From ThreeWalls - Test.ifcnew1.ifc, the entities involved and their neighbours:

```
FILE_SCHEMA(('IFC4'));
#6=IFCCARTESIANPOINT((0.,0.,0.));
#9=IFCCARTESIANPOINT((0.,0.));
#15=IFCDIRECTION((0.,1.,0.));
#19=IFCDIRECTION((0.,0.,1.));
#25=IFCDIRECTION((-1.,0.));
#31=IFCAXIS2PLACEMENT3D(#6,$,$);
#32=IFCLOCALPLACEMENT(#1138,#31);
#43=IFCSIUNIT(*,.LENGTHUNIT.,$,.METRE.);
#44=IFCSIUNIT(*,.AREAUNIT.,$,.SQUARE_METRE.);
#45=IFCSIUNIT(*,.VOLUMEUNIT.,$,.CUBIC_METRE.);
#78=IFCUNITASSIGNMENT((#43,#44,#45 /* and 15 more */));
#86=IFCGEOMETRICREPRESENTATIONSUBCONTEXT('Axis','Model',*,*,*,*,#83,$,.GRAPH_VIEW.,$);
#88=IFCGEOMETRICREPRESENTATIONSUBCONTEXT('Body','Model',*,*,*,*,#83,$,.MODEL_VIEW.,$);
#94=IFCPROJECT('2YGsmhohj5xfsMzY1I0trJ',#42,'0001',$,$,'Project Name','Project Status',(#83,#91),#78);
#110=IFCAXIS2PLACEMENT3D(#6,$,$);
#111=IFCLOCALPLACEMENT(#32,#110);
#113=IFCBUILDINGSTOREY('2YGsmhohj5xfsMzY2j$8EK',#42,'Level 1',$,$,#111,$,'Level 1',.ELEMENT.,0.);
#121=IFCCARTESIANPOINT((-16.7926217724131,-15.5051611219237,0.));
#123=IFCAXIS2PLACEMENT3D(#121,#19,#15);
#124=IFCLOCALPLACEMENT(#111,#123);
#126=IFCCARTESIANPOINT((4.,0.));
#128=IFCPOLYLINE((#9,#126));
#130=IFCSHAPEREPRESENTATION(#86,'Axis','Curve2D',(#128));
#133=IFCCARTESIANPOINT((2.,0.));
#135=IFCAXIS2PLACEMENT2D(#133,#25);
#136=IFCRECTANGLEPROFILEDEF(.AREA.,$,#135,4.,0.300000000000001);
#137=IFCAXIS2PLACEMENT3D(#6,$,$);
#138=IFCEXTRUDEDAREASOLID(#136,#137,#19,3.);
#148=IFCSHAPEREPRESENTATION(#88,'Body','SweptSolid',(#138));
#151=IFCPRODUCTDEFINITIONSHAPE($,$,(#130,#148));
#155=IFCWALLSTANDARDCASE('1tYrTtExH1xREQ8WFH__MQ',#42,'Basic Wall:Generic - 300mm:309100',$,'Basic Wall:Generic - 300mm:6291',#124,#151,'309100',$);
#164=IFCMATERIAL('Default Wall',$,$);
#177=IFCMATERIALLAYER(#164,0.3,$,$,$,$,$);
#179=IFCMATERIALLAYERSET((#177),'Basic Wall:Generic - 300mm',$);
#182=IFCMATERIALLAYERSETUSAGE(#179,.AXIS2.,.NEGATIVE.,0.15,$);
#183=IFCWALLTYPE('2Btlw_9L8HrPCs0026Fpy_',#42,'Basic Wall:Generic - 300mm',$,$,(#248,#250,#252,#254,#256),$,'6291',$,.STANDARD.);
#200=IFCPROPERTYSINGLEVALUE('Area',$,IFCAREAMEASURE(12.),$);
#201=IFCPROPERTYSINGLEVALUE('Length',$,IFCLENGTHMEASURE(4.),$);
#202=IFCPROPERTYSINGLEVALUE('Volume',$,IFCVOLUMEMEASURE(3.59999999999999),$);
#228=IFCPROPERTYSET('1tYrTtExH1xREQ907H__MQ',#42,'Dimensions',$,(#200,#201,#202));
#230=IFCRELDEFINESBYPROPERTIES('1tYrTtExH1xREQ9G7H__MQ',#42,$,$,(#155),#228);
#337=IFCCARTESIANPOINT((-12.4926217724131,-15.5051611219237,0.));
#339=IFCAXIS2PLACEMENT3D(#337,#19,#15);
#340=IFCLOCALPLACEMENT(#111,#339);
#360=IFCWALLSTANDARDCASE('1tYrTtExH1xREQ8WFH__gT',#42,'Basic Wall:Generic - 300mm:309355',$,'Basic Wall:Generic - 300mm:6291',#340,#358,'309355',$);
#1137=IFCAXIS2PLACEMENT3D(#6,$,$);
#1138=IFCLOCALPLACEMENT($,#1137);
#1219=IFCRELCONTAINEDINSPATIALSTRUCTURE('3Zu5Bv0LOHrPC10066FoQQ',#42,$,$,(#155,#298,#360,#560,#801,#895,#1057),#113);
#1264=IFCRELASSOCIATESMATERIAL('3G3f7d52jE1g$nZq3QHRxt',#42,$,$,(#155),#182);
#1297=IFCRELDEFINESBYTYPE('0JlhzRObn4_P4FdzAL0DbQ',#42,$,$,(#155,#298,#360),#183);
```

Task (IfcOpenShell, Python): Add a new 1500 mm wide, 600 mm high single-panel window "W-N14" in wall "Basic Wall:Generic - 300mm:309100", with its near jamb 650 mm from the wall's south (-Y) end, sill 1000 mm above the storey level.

```python
import numpy as np
import ifcopenshell
import ifcopenshell.api.feature
import ifcopenshell.api.geometry
import ifcopenshell.api.pset
import ifcopenshell.api.root
import ifcopenshell.api.spatial
import ifcopenshell.geom
import ifcopenshell.util.element
import ifcopenshell.util.placement
import ifcopenshell.util.representation
import ifcopenshell.util.shape
import ifcopenshell.util.unit

model = ifcopenshell.open("ThreeWalls - Test.ifcnew1.ifc")
unit_scale = ifcopenshell.util.unit.calculate_unit_scale(model)
area_scale = ifcopenshell.util.unit.calculate_unit_scale(model, "AREAUNIT")
volume_scale = ifcopenshell.util.unit.calculate_unit_scale(model, "VOLUMEUNIT")
settings = ifcopenshell.geom.settings()


def volume(element):
    """Net volume in cubic metres, openings subtracted."""
    shape = ifcopenshell.geom.create_shape(settings, element)
    return ifcopenshell.util.shape.get_volume(shape.geometry)


wall = model.by_guid("1tYrTtExH1xREQ8WFH__MQ")
storey = ifcopenshell.util.element.get_container(wall, ifc_class="IfcBuildingStorey")
context = ifcopenshell.util.representation.get_context(model, "Model", "Body", "MODEL_VIEW")
before = volume(wall)

width, height, from_end, sill = 1.5, 0.6, 0.65, 1  # metres

# The wall runs along its own X axis, and the end named is its -X end.
wall_shape = ifcopenshell.geom.create_shape(settings, wall)
x, y, z = ifcopenshell.util.shape.get_vertices(wall_shape.geometry).T
start = x.min() + from_end
face, thickness = float(y.min()), float(y.max() - y.min())
wall_matrix = ifcopenshell.util.placement.get_local_placement(wall.ObjectPlacement)
level = ifcopenshell.util.placement.get_local_placement(storey.ObjectPlacement)[2, 3]


def in_wall(x, y):
    """Placement at x, y metres in the wall's axes, at sill height."""
    matrix = wall_matrix.copy()
    matrix[:, 3] = wall_matrix @ np.array([x / unit_scale, y / unit_scale, 0.0, 1.0])
    matrix[2, 3] = level + sill / unit_scale
    return matrix


# Opening: a box that overshoots both wall faces by 50 mm.
opening = ifcopenshell.api.root.create_entity(model, ifc_class="IfcOpeningElement", predefined_type="OPENING")
box = ifcopenshell.api.geometry.add_wall_representation(
    model, context=context, length=width, height=height, thickness=thickness + 0.1
)
ifcopenshell.api.geometry.assign_representation(model, product=opening, representation=box)
ifcopenshell.api.geometry.edit_object_placement(model, product=opening, matrix=in_wall(start, face - 0.05), is_si=False)
ifcopenshell.api.feature.add_feature(model, feature=opening, element=wall)

window = ifcopenshell.api.root.create_entity(model, ifc_class="IfcWindow", name="W-N14", predefined_type="WINDOW")
window.OverallWidth, window.OverallHeight = width / unit_scale, height / unit_scale
window.PartitioningType = "SINGLE_PANEL"
body = ifcopenshell.api.geometry.add_window_representation(
    model,
    context=context,
    overall_width=window.OverallWidth,
    overall_height=window.OverallHeight,
    partition_type="SINGLE_PANEL",
)
ifcopenshell.api.geometry.assign_representation(model, product=window, representation=body)
ifcopenshell.api.spatial.assign_container(model, products=[window], relating_structure=storey)
ifcopenshell.api.feature.add_filling(model, opening=opening, element=window)

# Centre the window in the wall's thickness.
ifcopenshell.api.geometry.edit_object_placement(model, product=window, matrix=in_wall(start, face), is_si=False)
window_shape = ifcopenshell.geom.create_shape(settings, window)
depth = ifcopenshell.util.shape.get_vertices(window_shape.geometry)[:, 1]
offset = face + thickness / 2 - (depth.min() + depth.max()) / 2
ifcopenshell.api.geometry.edit_object_placement(model, product=window, matrix=in_wall(start, offset), is_si=False)

after = volume(wall)

# Update the wall's stored quantities.
pset = model.by_id(ifcopenshell.util.element.get_pset(wall, "Dimensions", should_inherit=False)["id"])
ifcopenshell.api.pset.edit_pset(model, pset=pset, properties={
    "Area": model.create_entity("IfcAreaMeasure", after / thickness / area_scale),
    "Volume": model.create_entity("IfcVolumeMeasure", after / volume_scale),
})

print(f"wall volume {before:.3f} -> {after:.3f} m3")

model.write("ThreeWalls - Test.ifcnew1_rev.ifc")
```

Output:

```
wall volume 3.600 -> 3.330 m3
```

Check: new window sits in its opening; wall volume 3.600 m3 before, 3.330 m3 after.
